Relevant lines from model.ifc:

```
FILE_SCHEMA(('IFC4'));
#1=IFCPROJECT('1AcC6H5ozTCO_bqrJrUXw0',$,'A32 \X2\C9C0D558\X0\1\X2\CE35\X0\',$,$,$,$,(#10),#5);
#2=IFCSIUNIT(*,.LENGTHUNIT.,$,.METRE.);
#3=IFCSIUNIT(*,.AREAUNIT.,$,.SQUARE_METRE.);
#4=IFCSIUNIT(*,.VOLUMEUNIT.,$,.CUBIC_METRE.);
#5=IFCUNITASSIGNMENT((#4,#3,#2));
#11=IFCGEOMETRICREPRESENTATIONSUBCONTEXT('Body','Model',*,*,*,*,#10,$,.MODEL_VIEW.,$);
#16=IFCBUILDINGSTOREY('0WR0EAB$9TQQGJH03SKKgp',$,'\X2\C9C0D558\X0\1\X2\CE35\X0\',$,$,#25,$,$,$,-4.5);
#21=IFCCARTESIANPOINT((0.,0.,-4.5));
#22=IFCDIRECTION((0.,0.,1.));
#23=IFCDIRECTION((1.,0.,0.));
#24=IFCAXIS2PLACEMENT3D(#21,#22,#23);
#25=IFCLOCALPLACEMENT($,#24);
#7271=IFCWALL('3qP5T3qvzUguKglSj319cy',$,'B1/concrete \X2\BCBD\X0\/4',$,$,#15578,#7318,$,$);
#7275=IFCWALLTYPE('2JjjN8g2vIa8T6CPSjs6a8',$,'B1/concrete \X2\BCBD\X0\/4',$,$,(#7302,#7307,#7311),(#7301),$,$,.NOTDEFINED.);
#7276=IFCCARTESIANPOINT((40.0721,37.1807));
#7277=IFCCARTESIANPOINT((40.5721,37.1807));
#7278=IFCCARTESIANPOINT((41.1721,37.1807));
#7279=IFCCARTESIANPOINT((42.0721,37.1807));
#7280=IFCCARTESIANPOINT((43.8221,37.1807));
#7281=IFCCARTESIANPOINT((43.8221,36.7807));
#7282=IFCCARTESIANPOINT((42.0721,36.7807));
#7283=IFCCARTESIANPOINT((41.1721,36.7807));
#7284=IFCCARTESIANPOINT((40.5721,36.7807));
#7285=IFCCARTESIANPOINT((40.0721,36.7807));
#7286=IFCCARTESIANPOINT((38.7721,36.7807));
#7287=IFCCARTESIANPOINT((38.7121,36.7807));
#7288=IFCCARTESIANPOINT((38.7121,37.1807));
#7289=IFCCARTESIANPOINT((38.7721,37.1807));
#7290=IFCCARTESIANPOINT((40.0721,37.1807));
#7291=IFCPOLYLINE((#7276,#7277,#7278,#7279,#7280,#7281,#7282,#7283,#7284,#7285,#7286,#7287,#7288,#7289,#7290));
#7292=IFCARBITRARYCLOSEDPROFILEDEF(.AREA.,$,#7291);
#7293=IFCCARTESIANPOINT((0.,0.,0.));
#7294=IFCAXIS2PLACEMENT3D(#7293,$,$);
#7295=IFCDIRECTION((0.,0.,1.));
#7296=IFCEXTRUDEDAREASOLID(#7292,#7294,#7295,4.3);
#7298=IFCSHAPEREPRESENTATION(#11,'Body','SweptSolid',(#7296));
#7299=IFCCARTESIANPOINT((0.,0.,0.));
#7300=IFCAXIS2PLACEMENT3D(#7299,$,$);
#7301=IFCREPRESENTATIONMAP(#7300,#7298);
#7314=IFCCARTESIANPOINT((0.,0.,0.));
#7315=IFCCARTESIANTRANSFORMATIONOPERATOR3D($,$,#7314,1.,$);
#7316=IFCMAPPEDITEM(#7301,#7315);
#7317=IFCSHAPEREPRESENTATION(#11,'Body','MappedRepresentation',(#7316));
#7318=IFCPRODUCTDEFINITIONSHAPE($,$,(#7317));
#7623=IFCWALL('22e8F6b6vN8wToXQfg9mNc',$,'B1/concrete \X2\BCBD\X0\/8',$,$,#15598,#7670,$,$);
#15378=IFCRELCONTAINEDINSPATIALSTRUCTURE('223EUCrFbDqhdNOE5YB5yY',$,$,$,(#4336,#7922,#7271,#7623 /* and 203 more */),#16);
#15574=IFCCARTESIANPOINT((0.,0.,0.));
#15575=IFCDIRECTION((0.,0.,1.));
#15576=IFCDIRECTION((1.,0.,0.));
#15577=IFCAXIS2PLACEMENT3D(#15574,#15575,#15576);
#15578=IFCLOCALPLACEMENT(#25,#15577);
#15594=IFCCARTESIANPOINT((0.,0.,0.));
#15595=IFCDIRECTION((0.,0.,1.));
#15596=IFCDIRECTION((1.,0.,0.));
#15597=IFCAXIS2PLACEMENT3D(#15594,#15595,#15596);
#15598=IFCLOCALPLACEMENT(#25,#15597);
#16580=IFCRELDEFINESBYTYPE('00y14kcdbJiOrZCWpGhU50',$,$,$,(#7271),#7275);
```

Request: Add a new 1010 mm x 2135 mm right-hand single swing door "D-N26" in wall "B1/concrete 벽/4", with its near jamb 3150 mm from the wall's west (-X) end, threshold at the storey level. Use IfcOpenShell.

```python
import numpy as np
import ifcopenshell
import ifcopenshell.api.feature
import ifcopenshell.api.geometry
import ifcopenshell.api.root
import ifcopenshell.api.spatial
import ifcopenshell.geom
import ifcopenshell.util.element
import ifcopenshell.util.placement
import ifcopenshell.util.representation
import ifcopenshell.util.shape
import ifcopenshell.util.unit

model = ifcopenshell.open("model.ifc")
unit_scale = ifcopenshell.util.unit.calculate_unit_scale(model)
settings = ifcopenshell.geom.settings()


def volume(element):
    """Net volume in cubic metres, openings subtracted."""
    shape = ifcopenshell.geom.create_shape(settings, element)
    return ifcopenshell.util.shape.get_volume(shape.geometry)


wall = model.by_guid("3qP5T3qvzUguKglSj319cy")
storey = ifcopenshell.util.element.get_container(wall, ifc_class="IfcBuildingStorey")
context = ifcopenshell.util.representation.get_context(model, "Model", "Body", "MODEL_VIEW")
before = volume(wall)

width, height, from_end, sill = 1.01, 2.135, 3.15, 0.0  # metres

# The wall runs along its own X axis, and the end named is its -X end.
wall_shape = ifcopenshell.geom.create_shape(settings, wall)
x, y, z = ifcopenshell.util.shape.get_vertices(wall_shape.geometry).T
start = x.min() + from_end
face, thickness = float(y.min()), float(y.max() - y.min())
wall_matrix = ifcopenshell.util.placement.get_local_placement(wall.ObjectPlacement)
level = ifcopenshell.util.placement.get_local_placement(storey.ObjectPlacement)[2, 3]


def in_wall(x, y):
    """Placement at x, y metres in the wall's axes, at sill height."""
    matrix = wall_matrix.copy()
    matrix[:, 3] = wall_matrix @ np.array([x / unit_scale, y / unit_scale, 0.0, 1.0])
    matrix[2, 3] = level + sill / unit_scale
    return matrix


# Opening: a box that overshoots both wall faces by 50 mm.
opening = ifcopenshell.api.root.create_entity(model, ifc_class="IfcOpeningElement", predefined_type="OPENING")
box = ifcopenshell.api.geometry.add_wall_representation(
    model, context=context, length=width, height=height, thickness=thickness + 0.1
)
ifcopenshell.api.geometry.assign_representation(model, product=opening, representation=box)
ifcopenshell.api.geometry.edit_object_placement(model, product=opening, matrix=in_wall(start, face - 0.05), is_si=False)
ifcopenshell.api.feature.add_feature(model, feature=opening, element=wall)

door = ifcopenshell.api.root.create_entity(model, ifc_class="IfcDoor", name="D-N26", predefined_type="DOOR")
door.OverallWidth, door.OverallHeight = width / unit_scale, height / unit_scale
door.OperationType = "SINGLE_SWING_RIGHT"
body = ifcopenshell.api.geometry.add_door_representation(
    model,
    context=context,
    overall_width=door.OverallWidth,
    overall_height=door.OverallHeight,
    operation_type="SINGLE_SWING_RIGHT",
    lining_properties={"LiningDepth": thickness / unit_scale, "ThresholdDepth": thickness / unit_scale},
)
ifcopenshell.api.geometry.assign_representation(model, product=door, representation=body)
ifcopenshell.api.spatial.assign_container(model, products=[door], relating_structure=storey)
ifcopenshell.api.feature.add_filling(model, opening=opening, element=door)

# The lining spans the wall, so the door starts at the wall face.
ifcopenshell.api.geometry.edit_object_placement(model, product=door, matrix=in_wall(start, face), is_si=False)

after = volume(wall)

print(f"wall volume {before:.3f} -> {after:.3f} m3")

model.write("model_edited.ifc")
```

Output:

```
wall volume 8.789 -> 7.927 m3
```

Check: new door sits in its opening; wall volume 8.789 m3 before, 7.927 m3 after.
